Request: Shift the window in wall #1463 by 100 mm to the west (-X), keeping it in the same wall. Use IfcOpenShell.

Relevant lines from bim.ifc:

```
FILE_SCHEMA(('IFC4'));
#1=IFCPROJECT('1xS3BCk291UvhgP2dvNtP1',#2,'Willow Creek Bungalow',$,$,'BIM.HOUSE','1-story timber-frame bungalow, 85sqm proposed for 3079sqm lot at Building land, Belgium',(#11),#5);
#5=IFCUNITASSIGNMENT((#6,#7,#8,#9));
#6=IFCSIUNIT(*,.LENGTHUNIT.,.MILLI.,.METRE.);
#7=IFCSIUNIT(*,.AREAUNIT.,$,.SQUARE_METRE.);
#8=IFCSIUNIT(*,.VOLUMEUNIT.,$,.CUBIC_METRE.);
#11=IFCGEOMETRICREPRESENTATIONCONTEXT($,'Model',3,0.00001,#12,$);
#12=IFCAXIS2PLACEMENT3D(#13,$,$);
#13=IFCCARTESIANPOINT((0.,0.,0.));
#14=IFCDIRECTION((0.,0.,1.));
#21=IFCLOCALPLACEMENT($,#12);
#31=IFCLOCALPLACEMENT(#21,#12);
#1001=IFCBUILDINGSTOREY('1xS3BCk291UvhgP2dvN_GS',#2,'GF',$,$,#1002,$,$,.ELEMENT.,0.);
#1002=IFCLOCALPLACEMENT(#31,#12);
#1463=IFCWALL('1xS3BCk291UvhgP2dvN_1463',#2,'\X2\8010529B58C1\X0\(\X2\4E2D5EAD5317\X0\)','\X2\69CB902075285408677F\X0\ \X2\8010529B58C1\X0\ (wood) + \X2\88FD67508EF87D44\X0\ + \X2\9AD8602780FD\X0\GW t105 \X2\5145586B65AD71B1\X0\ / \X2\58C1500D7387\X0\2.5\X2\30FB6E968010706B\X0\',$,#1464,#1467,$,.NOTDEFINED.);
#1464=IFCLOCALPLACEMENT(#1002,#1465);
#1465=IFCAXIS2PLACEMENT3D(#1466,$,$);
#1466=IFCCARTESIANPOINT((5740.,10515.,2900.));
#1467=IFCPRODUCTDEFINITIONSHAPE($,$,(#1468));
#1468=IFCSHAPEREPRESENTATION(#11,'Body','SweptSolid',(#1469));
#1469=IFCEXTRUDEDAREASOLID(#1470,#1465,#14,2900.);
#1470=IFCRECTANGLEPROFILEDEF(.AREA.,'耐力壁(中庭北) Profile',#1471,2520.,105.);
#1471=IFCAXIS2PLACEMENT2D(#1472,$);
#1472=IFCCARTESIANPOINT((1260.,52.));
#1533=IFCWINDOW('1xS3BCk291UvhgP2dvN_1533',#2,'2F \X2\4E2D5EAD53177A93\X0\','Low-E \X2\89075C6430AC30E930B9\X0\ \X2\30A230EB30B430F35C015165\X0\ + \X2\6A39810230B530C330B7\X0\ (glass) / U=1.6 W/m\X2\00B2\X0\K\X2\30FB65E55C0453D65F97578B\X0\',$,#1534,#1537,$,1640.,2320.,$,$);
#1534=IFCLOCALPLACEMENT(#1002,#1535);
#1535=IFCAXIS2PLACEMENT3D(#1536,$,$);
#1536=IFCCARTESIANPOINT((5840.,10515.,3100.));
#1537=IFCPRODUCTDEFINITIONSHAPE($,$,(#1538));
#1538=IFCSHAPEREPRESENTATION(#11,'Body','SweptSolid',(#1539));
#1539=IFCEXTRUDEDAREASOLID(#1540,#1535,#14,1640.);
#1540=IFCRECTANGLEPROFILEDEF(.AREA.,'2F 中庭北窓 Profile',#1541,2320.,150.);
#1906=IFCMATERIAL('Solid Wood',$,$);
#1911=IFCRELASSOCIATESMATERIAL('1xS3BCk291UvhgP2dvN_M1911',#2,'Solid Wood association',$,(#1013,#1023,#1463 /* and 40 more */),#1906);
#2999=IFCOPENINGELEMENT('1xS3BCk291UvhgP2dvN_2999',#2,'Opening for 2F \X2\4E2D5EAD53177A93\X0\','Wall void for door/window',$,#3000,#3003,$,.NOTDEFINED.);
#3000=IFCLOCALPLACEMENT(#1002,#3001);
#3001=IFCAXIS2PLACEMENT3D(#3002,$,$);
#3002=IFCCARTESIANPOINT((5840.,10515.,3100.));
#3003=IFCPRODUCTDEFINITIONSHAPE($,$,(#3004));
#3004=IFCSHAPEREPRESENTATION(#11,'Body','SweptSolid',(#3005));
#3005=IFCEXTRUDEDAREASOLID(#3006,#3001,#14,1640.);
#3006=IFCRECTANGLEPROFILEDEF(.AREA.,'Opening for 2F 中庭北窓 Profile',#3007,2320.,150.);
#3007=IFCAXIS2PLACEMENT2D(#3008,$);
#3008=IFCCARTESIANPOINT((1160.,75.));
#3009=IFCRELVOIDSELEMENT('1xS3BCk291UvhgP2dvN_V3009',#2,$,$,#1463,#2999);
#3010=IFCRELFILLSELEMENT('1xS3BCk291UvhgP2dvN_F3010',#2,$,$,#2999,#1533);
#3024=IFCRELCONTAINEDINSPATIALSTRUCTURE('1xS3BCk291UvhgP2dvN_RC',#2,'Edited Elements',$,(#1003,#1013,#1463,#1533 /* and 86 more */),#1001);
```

```python
import ifcopenshell
import ifcopenshell.api.geometry
import ifcopenshell.util.placement
import ifcopenshell.util.unit

model = ifcopenshell.open("bim.ifc")
unit_scale = ifcopenshell.util.unit.calculate_unit_scale(model)

window = model.by_guid("1xS3BCk291UvhgP2dvN_1533")
opening = window.FillsVoids[0].RelatingOpeningElement
wall = opening.VoidsElements[0].RelatingBuildingElement

wall_matrix = ifcopenshell.util.placement.get_local_placement(wall.ObjectPlacement)
shift = wall_matrix[:3, 0] * -0.1 / unit_scale
before = ifcopenshell.util.placement.get_local_placement(window.ObjectPlacement)[:3, 3].copy()

# The window is not placed relative to its opening, so move both.
for product in (opening, window):
    matrix = ifcopenshell.util.placement.get_local_placement(product.ObjectPlacement)
    matrix[:3, 3] += shift
    ifcopenshell.api.geometry.edit_object_placement(model, product=product, matrix=matrix, is_si=False)

after = ifcopenshell.util.placement.get_local_placement(window.ObjectPlacement)[:3, 3]
print("window moved by", (after - before).round(3) + 0.0)

model.write("bim_rev.ifc")
```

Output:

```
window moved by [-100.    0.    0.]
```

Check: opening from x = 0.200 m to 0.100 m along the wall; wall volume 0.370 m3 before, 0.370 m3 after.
